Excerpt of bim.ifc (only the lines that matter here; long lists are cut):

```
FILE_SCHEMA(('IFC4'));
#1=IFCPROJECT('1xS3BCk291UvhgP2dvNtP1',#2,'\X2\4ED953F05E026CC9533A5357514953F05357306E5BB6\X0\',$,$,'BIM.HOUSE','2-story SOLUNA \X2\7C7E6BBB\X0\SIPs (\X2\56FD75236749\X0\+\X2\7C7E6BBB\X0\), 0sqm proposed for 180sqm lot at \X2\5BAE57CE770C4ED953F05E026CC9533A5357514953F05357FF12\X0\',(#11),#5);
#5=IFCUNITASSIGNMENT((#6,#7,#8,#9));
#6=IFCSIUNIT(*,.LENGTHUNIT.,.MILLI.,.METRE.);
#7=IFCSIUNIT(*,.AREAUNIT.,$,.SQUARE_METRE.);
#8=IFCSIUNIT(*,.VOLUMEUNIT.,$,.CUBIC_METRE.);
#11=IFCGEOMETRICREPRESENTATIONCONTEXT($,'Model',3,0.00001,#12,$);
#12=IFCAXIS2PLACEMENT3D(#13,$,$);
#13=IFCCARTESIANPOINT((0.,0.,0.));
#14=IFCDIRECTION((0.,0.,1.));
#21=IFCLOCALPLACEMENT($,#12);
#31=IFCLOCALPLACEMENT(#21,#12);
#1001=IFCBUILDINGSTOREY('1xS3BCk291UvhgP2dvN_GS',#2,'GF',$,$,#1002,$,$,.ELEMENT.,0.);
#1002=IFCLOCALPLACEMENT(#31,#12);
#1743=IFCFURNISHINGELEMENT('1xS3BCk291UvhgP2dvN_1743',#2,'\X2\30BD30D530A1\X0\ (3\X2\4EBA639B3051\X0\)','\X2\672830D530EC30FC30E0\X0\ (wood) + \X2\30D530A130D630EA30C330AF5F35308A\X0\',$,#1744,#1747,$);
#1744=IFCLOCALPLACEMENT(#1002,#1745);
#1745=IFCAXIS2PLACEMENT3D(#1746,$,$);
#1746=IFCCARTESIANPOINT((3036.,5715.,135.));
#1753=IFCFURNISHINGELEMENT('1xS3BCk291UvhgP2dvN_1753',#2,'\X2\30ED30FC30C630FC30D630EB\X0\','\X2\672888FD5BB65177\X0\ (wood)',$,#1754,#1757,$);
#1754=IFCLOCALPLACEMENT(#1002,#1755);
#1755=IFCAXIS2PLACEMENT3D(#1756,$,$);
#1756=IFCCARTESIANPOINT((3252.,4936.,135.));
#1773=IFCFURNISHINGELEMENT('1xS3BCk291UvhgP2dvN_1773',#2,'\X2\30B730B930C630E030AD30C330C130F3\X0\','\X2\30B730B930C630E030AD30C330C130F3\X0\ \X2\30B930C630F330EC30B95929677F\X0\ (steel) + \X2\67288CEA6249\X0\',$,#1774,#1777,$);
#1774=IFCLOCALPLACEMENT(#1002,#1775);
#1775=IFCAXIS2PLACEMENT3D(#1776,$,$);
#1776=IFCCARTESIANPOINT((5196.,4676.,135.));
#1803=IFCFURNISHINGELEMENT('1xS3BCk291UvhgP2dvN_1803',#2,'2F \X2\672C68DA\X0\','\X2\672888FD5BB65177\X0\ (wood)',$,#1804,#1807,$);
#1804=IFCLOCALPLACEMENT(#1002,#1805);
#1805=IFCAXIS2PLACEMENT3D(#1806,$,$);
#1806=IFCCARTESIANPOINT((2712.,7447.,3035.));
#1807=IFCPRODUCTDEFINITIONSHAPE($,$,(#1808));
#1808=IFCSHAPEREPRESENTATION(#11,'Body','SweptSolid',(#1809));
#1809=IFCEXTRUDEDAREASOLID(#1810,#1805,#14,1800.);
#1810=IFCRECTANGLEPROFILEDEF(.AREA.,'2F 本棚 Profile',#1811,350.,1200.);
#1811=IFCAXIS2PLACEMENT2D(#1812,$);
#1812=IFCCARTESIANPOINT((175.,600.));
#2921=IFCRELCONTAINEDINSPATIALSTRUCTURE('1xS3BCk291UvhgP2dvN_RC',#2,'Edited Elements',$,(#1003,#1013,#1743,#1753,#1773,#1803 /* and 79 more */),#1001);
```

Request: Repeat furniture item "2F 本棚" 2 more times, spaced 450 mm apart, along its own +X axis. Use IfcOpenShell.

```python
import ifcopenshell
import ifcopenshell.api.geometry
import ifcopenshell.api.root
import ifcopenshell.util.element
import ifcopenshell.util.placement

model = ifcopenshell.open("bim.ifc")


def reuse_history(source, copy):
    """copy_class also copies each property set's owner history, people and application; keep the originals."""
    for rel in copy.IsDefinedBy:
        if rel.is_a("IfcRelDefinesByProperties") and (history := rel.RelatingPropertyDefinition.OwnerHistory):
            rel.RelatingPropertyDefinition.OwnerHistory = source.OwnerHistory
            ifcopenshell.util.element.remove_deep2(model, history)


source = model.by_id(1803)
base = ifcopenshell.util.placement.get_local_placement(source.ObjectPlacement)
step = base[:3, 0] * 450.0

for i in range(1, 3):
    copy = ifcopenshell.api.root.copy_class(model, product=source)
    copy.Representation = ifcopenshell.util.element.copy_deep(
        model, source.Representation, exclude=["IfcGeometricRepresentationContext", "IfcRepresentationMap"]
    )
    reuse_history(source, copy)
    matrix = base.copy()
    matrix[:3, 3] += i * step
    print("added at", matrix[:3, 3].round(3) + 0.0)
    ifcopenshell.api.geometry.edit_object_placement(model, product=copy, matrix=matrix, is_si=False)

model.write("bim_rev.ifc")
```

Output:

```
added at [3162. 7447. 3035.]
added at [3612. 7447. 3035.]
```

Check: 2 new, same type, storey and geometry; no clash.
